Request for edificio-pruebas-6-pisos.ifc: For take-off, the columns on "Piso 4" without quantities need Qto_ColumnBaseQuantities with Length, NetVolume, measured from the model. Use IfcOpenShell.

First a look at what the model holds.

```python
import ifcopenshell
import ifcopenshell.util.element
import ifcopenshell.util.unit

model = ifcopenshell.open("edificio-pruebas-6-pisos.ifc")
print(model.schema)
for unit_type in ("LENGTHUNIT", "AREAUNIT", "VOLUMEUNIT"):
    print(unit_type, ifcopenshell.util.unit.calculate_unit_scale(model, unit_type))
storey = next(s for s in model.by_type("IfcBuildingStorey") if s.Name == "Piso 4")
columns = [e for e in ifcopenshell.util.element.get_decomposition(storey) if e.is_a("IfcColumn")]
for e in sorted(columns, key=lambda e: e.id()):
    print(e.id(), e.is_a(), e.Name, list(ifcopenshell.util.element.get_psets(e, qtos_only=True)), sep=" | ")
```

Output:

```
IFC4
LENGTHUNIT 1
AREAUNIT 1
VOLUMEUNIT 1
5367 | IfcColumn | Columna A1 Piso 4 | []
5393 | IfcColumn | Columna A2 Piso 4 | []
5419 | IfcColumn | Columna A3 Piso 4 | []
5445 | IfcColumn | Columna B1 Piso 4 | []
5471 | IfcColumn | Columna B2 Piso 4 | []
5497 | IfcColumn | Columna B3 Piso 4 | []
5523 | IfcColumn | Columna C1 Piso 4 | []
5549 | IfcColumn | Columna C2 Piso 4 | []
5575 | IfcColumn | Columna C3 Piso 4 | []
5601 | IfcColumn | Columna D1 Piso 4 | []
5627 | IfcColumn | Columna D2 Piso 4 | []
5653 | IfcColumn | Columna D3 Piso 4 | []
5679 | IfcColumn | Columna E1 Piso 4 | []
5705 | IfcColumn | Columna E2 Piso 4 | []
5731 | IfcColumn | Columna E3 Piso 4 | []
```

```python
import ifcopenshell
import ifcopenshell.api.pset
import ifcopenshell.geom
import ifcopenshell.util.element
import ifcopenshell.util.shape
import ifcopenshell.util.unit

model = ifcopenshell.open("edificio-pruebas-6-pisos.ifc")
unit_scale = ifcopenshell.util.unit.calculate_unit_scale(model)
volume_scale = ifcopenshell.util.unit.calculate_unit_scale(model, "VOLUMEUNIT")
settings = ifcopenshell.geom.settings()

storey = next(s for s in model.by_type("IfcBuildingStorey") if s.Name == "Piso 4")
columns = [e for e in ifcopenshell.util.element.get_decomposition(storey) if e.is_a("IfcColumn")]

for e in sorted(columns, key=lambda e: e.id()):
    if ifcopenshell.util.element.get_psets(e, qtos_only=True, should_inherit=False):
        continue
    # Geometry comes back in metres, in the element's own axes.
    shape = ifcopenshell.geom.create_shape(settings, e)
    values = {
        "Length": ifcopenshell.util.shape.get_z(shape.geometry) / unit_scale,
        "NetVolume": ifcopenshell.util.shape.get_volume(shape.geometry) / volume_scale,
    }
    qto = ifcopenshell.api.pset.add_qto(model, product=e, name="Qto_ColumnBaseQuantities")
    ifcopenshell.api.pset.edit_qto(model, qto=qto, properties=values)
    print(e.id(), {k: round(v, 3) for k, v in values.items()})

model.write("edificio-pruebas-6-pisos-out.ifc")
```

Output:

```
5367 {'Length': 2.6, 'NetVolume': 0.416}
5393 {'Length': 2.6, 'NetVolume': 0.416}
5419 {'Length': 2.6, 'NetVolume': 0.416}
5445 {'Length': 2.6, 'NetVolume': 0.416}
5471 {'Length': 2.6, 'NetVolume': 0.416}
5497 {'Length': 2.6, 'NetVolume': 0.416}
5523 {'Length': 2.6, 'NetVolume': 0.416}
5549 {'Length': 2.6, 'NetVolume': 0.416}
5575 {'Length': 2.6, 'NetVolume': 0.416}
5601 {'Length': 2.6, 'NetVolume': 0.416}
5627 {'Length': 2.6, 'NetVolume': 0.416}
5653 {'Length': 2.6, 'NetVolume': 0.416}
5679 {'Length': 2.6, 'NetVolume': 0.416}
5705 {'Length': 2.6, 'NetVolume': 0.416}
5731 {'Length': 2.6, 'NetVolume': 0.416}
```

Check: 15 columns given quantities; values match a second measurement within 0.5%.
